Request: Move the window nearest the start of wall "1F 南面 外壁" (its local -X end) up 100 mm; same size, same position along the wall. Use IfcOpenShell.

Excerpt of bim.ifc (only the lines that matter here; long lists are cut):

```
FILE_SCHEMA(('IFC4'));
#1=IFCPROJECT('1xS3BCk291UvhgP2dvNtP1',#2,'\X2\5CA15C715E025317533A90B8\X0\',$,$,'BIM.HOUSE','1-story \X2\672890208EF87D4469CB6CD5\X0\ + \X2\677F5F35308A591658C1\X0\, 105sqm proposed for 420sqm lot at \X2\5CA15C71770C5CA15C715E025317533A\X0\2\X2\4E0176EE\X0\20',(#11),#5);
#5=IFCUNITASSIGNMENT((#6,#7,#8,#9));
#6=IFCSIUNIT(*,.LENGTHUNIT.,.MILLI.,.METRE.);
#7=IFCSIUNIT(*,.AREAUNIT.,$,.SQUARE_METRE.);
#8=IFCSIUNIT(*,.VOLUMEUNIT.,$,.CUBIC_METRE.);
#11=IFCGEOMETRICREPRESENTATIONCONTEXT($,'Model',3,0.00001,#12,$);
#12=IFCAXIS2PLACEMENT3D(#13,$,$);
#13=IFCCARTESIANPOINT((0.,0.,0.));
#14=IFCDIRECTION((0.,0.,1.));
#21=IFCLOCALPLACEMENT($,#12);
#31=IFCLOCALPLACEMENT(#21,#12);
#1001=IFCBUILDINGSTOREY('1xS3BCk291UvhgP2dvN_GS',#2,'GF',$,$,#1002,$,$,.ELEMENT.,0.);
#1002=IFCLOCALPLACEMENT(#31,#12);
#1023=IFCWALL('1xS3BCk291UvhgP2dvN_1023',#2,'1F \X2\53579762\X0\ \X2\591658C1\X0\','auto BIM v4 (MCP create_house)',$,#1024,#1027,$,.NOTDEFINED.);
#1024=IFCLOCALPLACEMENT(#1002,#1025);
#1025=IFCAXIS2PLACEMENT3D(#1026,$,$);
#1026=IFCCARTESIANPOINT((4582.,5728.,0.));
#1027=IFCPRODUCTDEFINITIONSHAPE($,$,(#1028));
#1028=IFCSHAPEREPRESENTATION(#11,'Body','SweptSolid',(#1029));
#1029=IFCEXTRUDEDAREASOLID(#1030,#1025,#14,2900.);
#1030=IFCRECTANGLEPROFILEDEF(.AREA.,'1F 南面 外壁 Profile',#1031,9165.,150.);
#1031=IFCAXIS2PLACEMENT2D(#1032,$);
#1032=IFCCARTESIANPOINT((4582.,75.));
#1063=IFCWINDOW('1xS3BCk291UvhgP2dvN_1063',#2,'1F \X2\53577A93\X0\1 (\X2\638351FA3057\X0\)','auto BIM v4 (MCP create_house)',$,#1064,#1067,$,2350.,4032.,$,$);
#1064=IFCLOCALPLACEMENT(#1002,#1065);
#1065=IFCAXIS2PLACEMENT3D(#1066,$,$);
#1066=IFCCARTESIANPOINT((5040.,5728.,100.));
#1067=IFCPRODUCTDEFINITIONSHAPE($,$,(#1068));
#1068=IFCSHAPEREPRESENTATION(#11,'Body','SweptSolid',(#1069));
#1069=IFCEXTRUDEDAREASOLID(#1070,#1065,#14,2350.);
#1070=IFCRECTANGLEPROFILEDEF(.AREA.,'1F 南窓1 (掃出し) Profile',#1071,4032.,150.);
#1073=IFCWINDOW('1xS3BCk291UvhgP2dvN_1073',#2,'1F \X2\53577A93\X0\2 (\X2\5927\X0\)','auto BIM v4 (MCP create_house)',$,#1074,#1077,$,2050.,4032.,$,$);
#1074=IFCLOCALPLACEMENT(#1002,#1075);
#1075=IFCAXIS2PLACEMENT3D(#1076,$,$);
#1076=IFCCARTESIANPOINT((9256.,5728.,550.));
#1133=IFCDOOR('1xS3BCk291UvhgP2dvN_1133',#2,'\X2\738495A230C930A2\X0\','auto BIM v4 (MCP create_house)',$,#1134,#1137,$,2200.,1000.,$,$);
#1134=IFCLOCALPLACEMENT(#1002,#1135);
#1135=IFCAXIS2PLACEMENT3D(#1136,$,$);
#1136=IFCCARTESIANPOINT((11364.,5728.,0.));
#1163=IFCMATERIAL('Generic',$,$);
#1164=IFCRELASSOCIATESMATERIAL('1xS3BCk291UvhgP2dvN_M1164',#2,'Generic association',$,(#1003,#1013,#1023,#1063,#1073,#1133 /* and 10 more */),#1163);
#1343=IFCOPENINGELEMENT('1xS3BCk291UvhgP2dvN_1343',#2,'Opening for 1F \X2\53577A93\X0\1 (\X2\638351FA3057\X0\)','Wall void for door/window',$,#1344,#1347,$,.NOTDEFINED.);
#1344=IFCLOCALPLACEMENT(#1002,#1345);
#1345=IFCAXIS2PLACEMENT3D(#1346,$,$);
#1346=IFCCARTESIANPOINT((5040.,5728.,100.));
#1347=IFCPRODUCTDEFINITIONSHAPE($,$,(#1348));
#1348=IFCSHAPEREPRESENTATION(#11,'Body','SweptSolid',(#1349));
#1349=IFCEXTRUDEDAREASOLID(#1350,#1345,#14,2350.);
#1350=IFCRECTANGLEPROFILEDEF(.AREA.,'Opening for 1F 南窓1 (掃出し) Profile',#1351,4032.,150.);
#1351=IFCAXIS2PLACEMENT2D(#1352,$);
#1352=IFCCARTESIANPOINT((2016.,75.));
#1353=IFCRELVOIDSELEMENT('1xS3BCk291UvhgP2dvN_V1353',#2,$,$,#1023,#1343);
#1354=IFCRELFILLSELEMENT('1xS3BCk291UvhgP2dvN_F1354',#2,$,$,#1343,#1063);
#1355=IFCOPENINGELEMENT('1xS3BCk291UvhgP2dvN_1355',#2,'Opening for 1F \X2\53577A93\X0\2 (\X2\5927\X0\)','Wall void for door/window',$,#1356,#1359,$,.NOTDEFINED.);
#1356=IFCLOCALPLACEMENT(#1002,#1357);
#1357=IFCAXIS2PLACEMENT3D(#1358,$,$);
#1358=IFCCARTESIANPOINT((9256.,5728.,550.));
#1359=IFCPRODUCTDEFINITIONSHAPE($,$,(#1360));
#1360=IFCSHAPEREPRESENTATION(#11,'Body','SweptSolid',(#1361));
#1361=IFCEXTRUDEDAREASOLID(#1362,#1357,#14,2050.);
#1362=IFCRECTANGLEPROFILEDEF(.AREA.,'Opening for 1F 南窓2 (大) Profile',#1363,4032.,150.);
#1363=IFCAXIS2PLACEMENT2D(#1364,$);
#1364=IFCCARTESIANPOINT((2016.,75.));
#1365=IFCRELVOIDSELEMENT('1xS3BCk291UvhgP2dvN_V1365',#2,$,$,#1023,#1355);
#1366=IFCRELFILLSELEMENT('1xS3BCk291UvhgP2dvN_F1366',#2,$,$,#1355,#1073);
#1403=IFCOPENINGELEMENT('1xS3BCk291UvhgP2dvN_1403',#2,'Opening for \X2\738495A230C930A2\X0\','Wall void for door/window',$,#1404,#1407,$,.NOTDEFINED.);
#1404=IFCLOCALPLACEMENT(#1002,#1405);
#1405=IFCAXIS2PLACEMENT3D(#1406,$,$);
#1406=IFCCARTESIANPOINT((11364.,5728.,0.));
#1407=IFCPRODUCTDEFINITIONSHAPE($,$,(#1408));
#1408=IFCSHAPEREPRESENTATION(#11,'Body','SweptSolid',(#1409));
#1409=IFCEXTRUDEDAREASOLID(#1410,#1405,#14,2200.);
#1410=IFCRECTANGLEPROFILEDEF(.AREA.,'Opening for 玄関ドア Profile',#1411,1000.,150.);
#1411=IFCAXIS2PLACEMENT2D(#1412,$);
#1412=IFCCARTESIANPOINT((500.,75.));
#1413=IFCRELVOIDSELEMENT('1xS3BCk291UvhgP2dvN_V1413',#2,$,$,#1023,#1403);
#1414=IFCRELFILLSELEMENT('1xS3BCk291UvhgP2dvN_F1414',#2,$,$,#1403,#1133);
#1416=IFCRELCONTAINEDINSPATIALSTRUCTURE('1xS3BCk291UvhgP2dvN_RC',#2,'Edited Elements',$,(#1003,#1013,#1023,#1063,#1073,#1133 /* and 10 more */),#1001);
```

```python
import numpy as np
import ifcopenshell
import ifcopenshell.api.geometry
import ifcopenshell.util.placement
import ifcopenshell.util.unit

model = ifcopenshell.open("bim.ifc")
unit_scale = ifcopenshell.util.unit.calculate_unit_scale(model)

window = model.by_guid("1xS3BCk291UvhgP2dvN_1063")
opening = window.FillsVoids[0].RelatingOpeningElement
dz = 100.0

shift = np.array([0.0, 0.0, dz])
# The window is not placed relative to its opening, so move both.
for product in (opening, window):
    matrix = ifcopenshell.util.placement.get_local_placement(product.ObjectPlacement)
    matrix[:3, 3] += shift
    ifcopenshell.api.geometry.edit_object_placement(model, product=product, matrix=matrix, is_si=False)

print(f"moved by {dz * unit_scale:+.3f} m")

model.write("bim_updated.ifc")
```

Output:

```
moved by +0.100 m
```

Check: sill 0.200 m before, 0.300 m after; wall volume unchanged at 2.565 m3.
